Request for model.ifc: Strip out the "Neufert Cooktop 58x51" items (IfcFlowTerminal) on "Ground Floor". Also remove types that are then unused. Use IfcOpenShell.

First a look at what the model holds.

```python
import ifcopenshell
import ifcopenshell.util.element

model = ifcopenshell.open("model.ifc")
print(model.schema)
storey = next(s for s in model.by_type("IfcBuildingStorey") if s.Name == "Ground Floor")
terminals = [e for e in ifcopenshell.util.element.get_decomposition(storey) if e.is_a("IfcFlowTerminal")]
seen = {}
for e in terminals:
    element_type = ifcopenshell.util.element.get_type(e)
    name = element_type.Name if element_type not in (None, e) else None
    seen[name] = seen.get(name, 0) + 1
for name, count in sorted(seen.items(), key=str):
    print(count, "x", name)
```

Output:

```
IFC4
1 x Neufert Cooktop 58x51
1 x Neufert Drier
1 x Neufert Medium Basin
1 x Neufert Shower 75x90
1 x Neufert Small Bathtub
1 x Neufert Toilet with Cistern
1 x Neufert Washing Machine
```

```python
import ifcopenshell
import ifcopenshell.api.root
import ifcopenshell.util.element

model = ifcopenshell.open("model.ifc")

storey = next(s for s in model.by_type("IfcBuildingStorey") if s.Name == "Ground Floor")
terminals = [e for e in ifcopenshell.util.element.get_decomposition(storey) if e.is_a("IfcFlowTerminal")]
targets = [e for e in terminals if (t := ifcopenshell.util.element.get_type(e)) not in (None, e) and t.Name == "Neufert Cooktop 58x51"]
types = {ifcopenshell.util.element.get_type(e) for e in targets} - {None, *targets}

for e in targets:
    ifcopenshell.api.root.remove_product(model, product=e)
print(len(targets), "removed")

unused = [t for t in types if not ifcopenshell.util.element.get_types(t)]
for t in unused:
    ifcopenshell.api.root.remove_product(model, product=t)
print(len(unused), "unused types removed")

model.write("model_v2.ifc")
```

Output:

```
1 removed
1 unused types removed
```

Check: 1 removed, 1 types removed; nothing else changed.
